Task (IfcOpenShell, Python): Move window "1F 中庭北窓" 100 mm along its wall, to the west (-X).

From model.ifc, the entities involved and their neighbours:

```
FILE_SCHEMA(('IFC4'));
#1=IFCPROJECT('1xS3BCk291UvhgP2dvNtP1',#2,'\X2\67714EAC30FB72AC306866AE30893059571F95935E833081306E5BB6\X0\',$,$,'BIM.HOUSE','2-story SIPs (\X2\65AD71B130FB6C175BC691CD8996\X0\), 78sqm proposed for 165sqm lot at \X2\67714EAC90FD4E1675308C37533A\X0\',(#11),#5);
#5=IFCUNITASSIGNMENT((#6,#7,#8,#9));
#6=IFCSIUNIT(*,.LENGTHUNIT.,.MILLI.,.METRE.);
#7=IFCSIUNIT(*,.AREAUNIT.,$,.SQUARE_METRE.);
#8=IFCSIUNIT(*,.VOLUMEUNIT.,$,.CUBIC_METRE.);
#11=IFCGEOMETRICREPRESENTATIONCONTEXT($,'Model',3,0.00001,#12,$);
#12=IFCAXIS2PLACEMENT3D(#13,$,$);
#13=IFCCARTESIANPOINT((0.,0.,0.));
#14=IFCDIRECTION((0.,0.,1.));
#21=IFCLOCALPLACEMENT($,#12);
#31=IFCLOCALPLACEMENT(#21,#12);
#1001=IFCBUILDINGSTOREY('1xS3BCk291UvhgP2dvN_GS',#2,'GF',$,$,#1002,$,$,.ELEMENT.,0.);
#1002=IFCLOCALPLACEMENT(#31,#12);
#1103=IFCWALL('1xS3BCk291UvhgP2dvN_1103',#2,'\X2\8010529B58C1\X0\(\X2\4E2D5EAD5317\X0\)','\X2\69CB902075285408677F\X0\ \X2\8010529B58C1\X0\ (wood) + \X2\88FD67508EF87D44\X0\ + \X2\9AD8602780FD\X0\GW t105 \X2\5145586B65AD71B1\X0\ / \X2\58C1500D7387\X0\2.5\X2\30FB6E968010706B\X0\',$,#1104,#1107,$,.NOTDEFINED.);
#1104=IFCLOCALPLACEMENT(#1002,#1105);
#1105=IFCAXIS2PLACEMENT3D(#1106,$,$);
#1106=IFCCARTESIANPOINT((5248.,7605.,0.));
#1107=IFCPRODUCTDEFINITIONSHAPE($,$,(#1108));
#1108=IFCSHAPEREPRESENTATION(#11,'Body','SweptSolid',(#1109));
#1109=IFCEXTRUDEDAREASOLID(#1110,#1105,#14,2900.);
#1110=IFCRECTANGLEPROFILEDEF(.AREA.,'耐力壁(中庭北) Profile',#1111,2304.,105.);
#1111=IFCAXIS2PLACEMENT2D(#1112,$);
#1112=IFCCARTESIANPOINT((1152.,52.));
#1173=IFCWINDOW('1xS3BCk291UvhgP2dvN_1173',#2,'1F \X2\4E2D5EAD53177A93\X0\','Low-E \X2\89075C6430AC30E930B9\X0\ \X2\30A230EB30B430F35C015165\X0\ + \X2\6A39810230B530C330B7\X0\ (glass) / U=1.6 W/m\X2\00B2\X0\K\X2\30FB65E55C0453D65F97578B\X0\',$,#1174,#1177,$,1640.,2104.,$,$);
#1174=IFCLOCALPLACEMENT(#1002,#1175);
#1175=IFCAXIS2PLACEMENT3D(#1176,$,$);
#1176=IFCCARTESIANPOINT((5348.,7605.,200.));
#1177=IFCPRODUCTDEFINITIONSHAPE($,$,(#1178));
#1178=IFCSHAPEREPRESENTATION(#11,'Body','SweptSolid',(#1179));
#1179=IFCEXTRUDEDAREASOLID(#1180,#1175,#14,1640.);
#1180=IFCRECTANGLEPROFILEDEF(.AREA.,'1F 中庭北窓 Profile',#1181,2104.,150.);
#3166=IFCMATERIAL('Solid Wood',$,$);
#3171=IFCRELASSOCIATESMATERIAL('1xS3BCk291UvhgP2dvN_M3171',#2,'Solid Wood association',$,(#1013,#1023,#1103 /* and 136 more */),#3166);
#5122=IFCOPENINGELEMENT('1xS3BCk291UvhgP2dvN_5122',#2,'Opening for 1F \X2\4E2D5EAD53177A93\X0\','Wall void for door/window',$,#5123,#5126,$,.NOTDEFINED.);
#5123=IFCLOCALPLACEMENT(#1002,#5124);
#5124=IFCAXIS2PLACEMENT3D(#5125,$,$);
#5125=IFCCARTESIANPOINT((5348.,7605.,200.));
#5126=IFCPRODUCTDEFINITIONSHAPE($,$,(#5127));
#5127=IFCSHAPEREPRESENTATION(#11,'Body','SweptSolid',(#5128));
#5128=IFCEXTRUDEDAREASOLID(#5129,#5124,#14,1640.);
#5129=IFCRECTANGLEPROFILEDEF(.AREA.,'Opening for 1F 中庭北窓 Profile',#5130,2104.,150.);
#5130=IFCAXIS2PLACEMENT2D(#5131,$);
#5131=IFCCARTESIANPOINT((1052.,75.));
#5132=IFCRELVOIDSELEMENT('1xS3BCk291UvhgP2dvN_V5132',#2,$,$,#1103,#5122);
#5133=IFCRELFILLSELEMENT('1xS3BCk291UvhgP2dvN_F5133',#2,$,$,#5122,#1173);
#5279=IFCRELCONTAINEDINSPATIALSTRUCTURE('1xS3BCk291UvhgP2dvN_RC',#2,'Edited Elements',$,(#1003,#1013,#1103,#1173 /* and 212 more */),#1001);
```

```python
import ifcopenshell
import ifcopenshell.api.geometry
import ifcopenshell.util.placement

model = ifcopenshell.open("model.ifc")

window = model.by_id(1173)
opening = window.FillsVoids[0].RelatingOpeningElement
wall = opening.VoidsElements[0].RelatingBuildingElement

wall_matrix = ifcopenshell.util.placement.get_local_placement(wall.ObjectPlacement)
shift = wall_matrix[:3, 0] * -100.0
before = ifcopenshell.util.placement.get_local_placement(window.ObjectPlacement)[:3, 3].copy()

# The window is not placed relative to its opening, so move both.
for product in (opening, window):
    matrix = ifcopenshell.util.placement.get_local_placement(product.ObjectPlacement)
    matrix[:3, 3] += shift
    ifcopenshell.api.geometry.edit_object_placement(model, product=product, matrix=matrix, is_si=False)

after = ifcopenshell.util.placement.get_local_placement(window.ObjectPlacement)[:3, 3]
print("window moved by", (after - before).round(3) + 0.0)

model.write("model_updated.ifc")
```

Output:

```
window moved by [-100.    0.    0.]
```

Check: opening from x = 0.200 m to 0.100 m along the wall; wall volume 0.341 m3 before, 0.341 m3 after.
